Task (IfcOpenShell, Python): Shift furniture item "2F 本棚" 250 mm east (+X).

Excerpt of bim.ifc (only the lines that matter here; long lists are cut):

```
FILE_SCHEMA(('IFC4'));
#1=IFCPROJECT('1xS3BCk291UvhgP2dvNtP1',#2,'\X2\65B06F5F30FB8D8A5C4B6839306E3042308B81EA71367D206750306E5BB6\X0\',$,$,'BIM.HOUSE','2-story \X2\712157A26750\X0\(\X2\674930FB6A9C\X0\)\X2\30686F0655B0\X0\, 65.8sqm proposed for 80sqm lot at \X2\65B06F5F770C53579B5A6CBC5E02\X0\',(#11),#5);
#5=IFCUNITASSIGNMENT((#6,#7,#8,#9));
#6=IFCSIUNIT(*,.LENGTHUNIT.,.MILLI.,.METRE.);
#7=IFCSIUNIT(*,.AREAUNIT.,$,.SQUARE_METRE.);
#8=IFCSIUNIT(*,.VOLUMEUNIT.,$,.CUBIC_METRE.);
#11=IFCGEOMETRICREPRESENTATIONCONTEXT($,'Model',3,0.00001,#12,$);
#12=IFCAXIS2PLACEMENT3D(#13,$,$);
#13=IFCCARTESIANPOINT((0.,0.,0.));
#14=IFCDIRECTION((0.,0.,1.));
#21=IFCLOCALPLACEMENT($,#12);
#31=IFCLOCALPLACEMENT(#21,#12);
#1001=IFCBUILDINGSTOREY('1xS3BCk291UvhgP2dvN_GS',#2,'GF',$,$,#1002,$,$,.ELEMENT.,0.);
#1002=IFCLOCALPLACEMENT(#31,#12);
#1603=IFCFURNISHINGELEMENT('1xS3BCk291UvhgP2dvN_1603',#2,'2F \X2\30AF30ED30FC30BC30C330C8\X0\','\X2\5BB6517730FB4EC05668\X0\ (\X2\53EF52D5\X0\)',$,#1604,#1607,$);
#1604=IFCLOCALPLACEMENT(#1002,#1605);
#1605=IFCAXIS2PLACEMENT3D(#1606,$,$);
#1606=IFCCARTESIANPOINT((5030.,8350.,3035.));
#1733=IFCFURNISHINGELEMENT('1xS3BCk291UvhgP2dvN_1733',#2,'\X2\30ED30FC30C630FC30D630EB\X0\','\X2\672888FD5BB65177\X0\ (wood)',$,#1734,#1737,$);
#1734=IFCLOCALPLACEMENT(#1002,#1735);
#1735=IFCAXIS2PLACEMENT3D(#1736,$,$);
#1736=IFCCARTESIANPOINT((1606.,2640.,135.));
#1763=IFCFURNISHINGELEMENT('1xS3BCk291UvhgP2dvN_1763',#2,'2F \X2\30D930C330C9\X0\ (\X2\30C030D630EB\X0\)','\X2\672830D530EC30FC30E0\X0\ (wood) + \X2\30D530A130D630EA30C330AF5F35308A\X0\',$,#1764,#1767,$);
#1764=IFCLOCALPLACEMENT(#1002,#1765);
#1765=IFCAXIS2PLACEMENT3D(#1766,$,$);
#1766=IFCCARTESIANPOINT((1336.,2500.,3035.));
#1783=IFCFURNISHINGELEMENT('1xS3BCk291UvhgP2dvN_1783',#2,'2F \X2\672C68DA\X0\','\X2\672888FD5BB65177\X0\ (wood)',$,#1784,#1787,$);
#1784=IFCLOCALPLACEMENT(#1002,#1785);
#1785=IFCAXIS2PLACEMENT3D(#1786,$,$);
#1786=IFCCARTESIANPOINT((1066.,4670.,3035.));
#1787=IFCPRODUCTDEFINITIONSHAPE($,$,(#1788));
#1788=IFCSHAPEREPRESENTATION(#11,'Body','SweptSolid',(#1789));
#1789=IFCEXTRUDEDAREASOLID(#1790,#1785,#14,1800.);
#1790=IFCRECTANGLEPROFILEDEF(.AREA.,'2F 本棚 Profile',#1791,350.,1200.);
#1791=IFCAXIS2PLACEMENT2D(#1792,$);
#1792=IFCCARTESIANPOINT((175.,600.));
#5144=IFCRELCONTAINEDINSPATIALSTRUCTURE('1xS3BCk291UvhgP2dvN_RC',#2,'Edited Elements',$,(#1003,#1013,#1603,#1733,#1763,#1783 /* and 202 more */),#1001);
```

```python
import ifcopenshell
import ifcopenshell.api.geometry
import ifcopenshell.util.placement

model = ifcopenshell.open("bim.ifc")

item = model.by_guid("1xS3BCk291UvhgP2dvN_1783")
matrix = ifcopenshell.util.placement.get_local_placement(item.ObjectPlacement)
matrix[0, 3] += 250.0
ifcopenshell.api.geometry.edit_object_placement(model, product=item, matrix=matrix, is_si=False)

print(ifcopenshell.util.placement.get_local_placement(item.ObjectPlacement).round(3) + 0.0)

model.write("bim_rev.ifc")
```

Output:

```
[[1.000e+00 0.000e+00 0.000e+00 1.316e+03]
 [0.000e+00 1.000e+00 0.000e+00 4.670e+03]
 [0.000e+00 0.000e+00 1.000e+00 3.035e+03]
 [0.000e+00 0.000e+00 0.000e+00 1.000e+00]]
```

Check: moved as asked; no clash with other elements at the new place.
